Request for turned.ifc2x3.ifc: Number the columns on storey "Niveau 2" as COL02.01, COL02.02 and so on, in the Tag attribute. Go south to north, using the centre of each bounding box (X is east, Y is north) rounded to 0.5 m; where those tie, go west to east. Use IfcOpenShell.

First a look at what the model holds.

```python
import ifcopenshell
import ifcopenshell.util.element
import ifcopenshell.util.placement

model = ifcopenshell.open("turned.ifc2x3.ifc")
print(model.schema)
storey = next(s for s in model.by_type("IfcBuildingStorey") if s.Name == "Niveau 2")
columns = [e for e in ifcopenshell.util.element.get_decomposition(storey) if e.is_a("IfcColumn")]
for e in sorted(columns, key=lambda e: e.id()):
    origin = ifcopenshell.util.placement.get_local_placement(e.ObjectPlacement)[:3, 3]
    print(e.id(), e.Tag, e.Name, origin.round(2) + 0.0, sep=" | ")
```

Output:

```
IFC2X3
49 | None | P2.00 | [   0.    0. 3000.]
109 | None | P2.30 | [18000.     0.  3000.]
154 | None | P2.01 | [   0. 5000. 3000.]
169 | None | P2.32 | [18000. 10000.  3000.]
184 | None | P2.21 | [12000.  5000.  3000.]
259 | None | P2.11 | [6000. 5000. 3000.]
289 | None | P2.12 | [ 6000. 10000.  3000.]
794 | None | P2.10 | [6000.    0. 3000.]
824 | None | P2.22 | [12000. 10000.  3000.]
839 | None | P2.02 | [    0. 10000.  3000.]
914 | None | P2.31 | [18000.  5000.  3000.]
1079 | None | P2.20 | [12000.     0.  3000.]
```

```python
import ifcopenshell
import ifcopenshell.geom
import ifcopenshell.util.element
import ifcopenshell.util.shape

model = ifcopenshell.open("turned.ifc2x3.ifc")
settings = ifcopenshell.geom.settings()
settings.set("use-world-coords", True)


def centre(element):
    shape = ifcopenshell.geom.create_shape(settings, element)
    return ifcopenshell.util.shape.get_bbox_centroid(shape.geometry)


storey = next(s for s in model.by_type("IfcBuildingStorey") if s.Name == "Niveau 2")
columns = [e for e in ifcopenshell.util.element.get_decomposition(storey) if e.is_a("IfcColumn")]

# Insertion points can sit at a corner or the storey origin, so sort by the geometry (in metres).
centres = {e: centre(e) for e in columns}
columns.sort(key=lambda e: (round(centres[e][1] / 0.5), centres[e][0]))

for i, e in enumerate(columns, start=1):
    number = f"COL02.{i:02d}"
    e.Tag = number
    print(e.id(), number)

model.write("turned.ifc2x3_v2.ifc")
```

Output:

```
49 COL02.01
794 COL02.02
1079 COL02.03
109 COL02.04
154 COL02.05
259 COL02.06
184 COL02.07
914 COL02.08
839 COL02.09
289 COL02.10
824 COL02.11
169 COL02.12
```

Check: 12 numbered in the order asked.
